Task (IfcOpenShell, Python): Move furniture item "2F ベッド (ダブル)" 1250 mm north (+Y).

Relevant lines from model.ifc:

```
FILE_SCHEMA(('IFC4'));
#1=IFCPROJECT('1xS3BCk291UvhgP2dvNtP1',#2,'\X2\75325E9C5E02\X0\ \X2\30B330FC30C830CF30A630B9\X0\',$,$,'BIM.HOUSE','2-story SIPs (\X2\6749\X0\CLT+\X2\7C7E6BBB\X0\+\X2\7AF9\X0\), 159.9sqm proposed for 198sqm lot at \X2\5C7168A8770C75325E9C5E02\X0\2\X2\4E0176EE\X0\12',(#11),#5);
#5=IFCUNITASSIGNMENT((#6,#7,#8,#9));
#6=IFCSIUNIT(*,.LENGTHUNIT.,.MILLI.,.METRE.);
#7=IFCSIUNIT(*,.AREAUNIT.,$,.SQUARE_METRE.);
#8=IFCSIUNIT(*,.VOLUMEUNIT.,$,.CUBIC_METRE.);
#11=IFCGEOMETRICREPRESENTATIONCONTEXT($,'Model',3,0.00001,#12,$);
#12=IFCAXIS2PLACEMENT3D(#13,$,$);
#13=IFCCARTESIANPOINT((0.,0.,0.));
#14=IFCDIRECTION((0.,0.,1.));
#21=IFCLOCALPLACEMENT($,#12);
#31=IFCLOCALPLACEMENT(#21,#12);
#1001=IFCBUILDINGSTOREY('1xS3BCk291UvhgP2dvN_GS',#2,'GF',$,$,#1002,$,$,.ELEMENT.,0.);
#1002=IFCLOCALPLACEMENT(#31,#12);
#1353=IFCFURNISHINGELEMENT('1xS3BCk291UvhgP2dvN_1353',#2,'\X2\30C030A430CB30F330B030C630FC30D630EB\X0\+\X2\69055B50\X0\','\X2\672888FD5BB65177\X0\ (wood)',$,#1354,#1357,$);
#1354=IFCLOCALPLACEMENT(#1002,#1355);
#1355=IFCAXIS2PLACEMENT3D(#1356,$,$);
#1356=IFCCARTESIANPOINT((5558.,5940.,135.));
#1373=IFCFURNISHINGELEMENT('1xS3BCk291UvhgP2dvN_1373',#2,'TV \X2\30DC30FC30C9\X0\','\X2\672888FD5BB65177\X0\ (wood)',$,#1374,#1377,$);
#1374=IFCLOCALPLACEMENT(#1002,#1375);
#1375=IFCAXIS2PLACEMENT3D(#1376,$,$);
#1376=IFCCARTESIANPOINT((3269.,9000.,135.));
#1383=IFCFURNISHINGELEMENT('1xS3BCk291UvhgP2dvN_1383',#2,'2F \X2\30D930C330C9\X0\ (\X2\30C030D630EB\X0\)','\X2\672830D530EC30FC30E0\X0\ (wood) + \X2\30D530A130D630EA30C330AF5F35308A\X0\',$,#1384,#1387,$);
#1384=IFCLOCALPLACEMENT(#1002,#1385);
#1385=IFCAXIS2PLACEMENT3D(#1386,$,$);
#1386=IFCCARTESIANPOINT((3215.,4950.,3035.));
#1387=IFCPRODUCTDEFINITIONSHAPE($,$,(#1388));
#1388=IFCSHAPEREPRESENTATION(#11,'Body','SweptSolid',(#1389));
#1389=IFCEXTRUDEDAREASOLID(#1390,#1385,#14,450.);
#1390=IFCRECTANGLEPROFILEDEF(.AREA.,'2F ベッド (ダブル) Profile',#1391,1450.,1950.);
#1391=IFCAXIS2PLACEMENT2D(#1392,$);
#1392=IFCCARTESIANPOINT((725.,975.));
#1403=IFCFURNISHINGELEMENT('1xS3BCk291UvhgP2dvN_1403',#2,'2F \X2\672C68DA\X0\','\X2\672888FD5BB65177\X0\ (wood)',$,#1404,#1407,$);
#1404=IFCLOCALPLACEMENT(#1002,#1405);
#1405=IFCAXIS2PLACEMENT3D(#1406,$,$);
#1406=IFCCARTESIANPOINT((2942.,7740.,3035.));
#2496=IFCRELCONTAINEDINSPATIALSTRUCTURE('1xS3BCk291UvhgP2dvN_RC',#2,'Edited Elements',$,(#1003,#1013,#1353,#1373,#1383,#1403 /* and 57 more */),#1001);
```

```python
import ifcopenshell
import ifcopenshell.api.geometry
import ifcopenshell.util.placement
import ifcopenshell.util.unit

model = ifcopenshell.open("model.ifc")
unit_scale = ifcopenshell.util.unit.calculate_unit_scale(model)

item = model.by_id(1383)
matrix = ifcopenshell.util.placement.get_local_placement(item.ObjectPlacement)
matrix[1, 3] += 1.25 / unit_scale
ifcopenshell.api.geometry.edit_object_placement(model, product=item, matrix=matrix, is_si=False)

print(ifcopenshell.util.placement.get_local_placement(item.ObjectPlacement).round(3) + 0.0)

model.write("model_updated.ifc")
```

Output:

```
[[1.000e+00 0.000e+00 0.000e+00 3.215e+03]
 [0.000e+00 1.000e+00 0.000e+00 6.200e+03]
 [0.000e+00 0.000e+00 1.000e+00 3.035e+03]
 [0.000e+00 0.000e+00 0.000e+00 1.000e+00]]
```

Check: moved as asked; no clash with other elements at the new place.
